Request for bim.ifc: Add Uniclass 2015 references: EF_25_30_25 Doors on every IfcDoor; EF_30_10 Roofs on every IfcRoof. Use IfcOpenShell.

First a look at what the model holds.

```python
import ifcopenshell

model = ifcopenshell.open("bim.ifc")
print(model.schema)
print("classifications:", [c.Name for c in model.by_type("IfcClassification")])
for ifc_class in ("IfcDoor", "IfcRoof", "IfcStair", "IfcWall", "IfcWindow"):
    print(ifc_class, len(model.by_type(ifc_class)))
```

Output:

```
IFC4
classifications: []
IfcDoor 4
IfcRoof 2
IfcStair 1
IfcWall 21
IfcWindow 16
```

```python
import ifcopenshell
import ifcopenshell.api.classification

model = ifcopenshell.open("bim.ifc")

system = ifcopenshell.api.classification.add_classification(model, classification="Uniclass 2015")

codes = {
    "IfcDoor": ("EF_25_30_25", "Doors"),
    "IfcRoof": ("EF_30_10", "Roofs"),
}
for ifc_class, (code, name) in codes.items():
    products = model.by_type(ifc_class)
    ifcopenshell.api.classification.add_reference(
        model, products=products, classification=system, identification=code, name=name
    )
    print(code, len(products))

model.write("bim_v2.ifc")
```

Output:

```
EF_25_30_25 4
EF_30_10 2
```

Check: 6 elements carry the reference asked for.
